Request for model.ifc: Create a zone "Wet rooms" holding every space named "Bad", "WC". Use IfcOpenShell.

First a look at what the model holds.

```python
import ifcopenshell

model = ifcopenshell.open("model.ifc")
print(model.schema)
seen = {}
for space in model.by_type("IfcSpace"):
    seen[space.LongName] = seen.get(space.LongName, 0) + 1
for name, count in sorted(seen.items(), key=str):
    print(count, "x", name)
print("zones:", [z.Name for z in model.by_type("IfcZone")][:20])
```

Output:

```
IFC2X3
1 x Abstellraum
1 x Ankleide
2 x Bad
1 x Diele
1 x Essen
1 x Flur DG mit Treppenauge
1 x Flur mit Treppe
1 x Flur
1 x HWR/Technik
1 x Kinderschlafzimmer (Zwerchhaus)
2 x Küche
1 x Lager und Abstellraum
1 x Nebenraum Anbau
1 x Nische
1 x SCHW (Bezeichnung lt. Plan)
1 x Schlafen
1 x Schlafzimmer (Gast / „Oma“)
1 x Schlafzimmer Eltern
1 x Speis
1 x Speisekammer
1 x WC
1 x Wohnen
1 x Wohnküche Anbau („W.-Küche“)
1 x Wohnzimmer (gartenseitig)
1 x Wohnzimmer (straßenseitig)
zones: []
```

```python
import ifcopenshell
import ifcopenshell.api.group
import ifcopenshell.api.root

model = ifcopenshell.open("model.ifc")

names = {"Bad", "WC"}
spaces = [s for s in model.by_type("IfcSpace") if s.LongName in names]

zone = ifcopenshell.api.root.create_entity(model, ifc_class="IfcZone", name="Wet rooms")
ifcopenshell.api.group.assign_group(model, products=spaces, group=zone)
print(len(spaces), "spaces in", zone.Name)

model.write("model_edited.ifc")
```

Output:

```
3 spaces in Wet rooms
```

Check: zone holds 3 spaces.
